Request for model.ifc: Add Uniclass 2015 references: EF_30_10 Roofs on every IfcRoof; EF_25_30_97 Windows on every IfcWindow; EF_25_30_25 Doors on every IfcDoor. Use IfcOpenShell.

First a look at what the model holds.

```python
import ifcopenshell

model = ifcopenshell.open("model.ifc")
print(model.schema)
print("classifications:", [c.Name for c in model.by_type("IfcClassification")])
for ifc_class in ("IfcDoor", "IfcRoof", "IfcStair", "IfcWall", "IfcWindow"):
    print(ifc_class, len(model.by_type(ifc_class)))
```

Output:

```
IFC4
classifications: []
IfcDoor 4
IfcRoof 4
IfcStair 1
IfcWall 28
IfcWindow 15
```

```python
import ifcopenshell
import ifcopenshell.api.classification

model = ifcopenshell.open("model.ifc")

system = ifcopenshell.api.classification.add_classification(model, classification="Uniclass 2015")

codes = {
    "IfcRoof": ("EF_30_10", "Roofs"),
    "IfcWindow": ("EF_25_30_97", "Windows"),
    "IfcDoor": ("EF_25_30_25", "Doors"),
}
for ifc_class, (code, name) in codes.items():
    products = model.by_type(ifc_class)
    ifcopenshell.api.classification.add_reference(
        model, products=products, classification=system, identification=code, name=name
    )
    print(code, len(products))

model.write("model_v2.ifc")
```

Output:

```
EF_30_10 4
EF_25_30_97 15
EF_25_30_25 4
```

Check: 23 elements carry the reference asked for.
